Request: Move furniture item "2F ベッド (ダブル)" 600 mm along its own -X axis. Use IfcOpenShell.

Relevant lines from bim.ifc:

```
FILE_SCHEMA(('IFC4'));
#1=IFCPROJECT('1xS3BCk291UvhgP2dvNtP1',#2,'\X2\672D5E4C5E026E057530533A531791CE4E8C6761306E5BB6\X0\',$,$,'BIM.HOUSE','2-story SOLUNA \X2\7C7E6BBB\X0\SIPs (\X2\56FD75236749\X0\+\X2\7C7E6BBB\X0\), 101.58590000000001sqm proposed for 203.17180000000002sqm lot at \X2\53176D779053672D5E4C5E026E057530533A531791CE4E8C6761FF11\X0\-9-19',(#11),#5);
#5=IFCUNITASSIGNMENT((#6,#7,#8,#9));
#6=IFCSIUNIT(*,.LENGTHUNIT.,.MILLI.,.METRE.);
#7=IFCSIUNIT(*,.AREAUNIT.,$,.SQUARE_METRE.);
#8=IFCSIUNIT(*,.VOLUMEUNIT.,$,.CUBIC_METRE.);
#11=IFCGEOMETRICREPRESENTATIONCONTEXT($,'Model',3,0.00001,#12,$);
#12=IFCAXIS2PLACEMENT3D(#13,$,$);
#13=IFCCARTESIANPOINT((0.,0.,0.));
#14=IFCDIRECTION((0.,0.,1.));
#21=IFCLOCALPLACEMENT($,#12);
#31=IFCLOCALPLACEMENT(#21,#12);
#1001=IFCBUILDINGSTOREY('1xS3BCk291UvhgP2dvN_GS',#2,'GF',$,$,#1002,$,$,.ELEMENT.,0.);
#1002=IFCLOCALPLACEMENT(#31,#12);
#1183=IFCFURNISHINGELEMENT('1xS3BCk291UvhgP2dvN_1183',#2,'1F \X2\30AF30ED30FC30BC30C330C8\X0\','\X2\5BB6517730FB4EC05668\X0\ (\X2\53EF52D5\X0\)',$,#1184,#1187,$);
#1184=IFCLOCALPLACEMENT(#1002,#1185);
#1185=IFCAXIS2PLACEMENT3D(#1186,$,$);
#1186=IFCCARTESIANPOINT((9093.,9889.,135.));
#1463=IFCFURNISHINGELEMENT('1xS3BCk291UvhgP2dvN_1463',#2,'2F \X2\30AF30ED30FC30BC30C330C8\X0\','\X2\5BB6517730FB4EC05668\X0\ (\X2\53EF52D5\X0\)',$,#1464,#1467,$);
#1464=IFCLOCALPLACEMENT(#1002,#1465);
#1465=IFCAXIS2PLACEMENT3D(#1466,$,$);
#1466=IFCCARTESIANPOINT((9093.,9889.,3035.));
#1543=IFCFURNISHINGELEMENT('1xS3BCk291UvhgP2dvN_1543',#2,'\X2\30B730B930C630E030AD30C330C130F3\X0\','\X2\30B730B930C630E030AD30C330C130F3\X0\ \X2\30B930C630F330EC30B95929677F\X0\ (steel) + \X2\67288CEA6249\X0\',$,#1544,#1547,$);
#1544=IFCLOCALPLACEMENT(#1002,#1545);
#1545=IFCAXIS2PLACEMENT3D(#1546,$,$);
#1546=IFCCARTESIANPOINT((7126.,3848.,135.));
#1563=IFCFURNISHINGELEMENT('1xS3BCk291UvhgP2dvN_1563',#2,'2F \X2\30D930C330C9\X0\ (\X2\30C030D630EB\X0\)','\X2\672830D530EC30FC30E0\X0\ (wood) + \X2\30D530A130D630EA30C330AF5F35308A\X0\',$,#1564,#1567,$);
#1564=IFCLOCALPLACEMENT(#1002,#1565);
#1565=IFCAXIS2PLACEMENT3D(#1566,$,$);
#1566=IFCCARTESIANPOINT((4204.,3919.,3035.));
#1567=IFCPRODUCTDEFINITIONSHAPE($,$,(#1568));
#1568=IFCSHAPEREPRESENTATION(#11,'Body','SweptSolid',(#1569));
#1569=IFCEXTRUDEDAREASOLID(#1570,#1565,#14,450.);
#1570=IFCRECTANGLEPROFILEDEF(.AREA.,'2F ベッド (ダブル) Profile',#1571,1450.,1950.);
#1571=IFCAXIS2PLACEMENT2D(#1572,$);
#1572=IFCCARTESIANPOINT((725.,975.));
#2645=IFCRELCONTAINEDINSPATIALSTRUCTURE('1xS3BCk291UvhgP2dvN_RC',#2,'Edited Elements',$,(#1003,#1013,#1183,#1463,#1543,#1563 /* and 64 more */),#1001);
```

```python
import ifcopenshell
import ifcopenshell.api.geometry
import ifcopenshell.util.placement

model = ifcopenshell.open("bim.ifc")

item = model.by_id(1563)
matrix = ifcopenshell.util.placement.get_local_placement(item.ObjectPlacement)
matrix[:3, 3] -= matrix[:3, 0] * 600.0
ifcopenshell.api.geometry.edit_object_placement(model, product=item, matrix=matrix, is_si=False)

print(ifcopenshell.util.placement.get_local_placement(item.ObjectPlacement).round(3) + 0.0)

model.write("bim_rev.ifc")
```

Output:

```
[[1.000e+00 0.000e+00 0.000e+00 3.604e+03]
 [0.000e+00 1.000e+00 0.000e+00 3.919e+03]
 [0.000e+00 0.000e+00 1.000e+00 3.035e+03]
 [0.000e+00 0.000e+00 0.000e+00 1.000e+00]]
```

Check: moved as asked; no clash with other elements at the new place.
